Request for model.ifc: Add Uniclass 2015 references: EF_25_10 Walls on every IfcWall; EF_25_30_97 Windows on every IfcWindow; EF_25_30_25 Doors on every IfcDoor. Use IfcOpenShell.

First a look at what the model holds.

```python
import ifcopenshell

model = ifcopenshell.open("model.ifc")
print(model.schema)
print("classifications:", [c.Name for c in model.by_type("IfcClassification")])
for ifc_class in ("IfcDoor", "IfcRoof", "IfcStair", "IfcWall", "IfcWindow"):
    print(ifc_class, len(model.by_type(ifc_class)))
```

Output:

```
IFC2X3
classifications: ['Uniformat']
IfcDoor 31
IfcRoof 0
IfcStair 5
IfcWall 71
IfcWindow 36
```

```python
import ifcopenshell
import ifcopenshell.api.classification

model = ifcopenshell.open("model.ifc")

# IFC2X3 requires Source and Edition and has no link from the project to the system.
system = model.create_entity("IfcClassification", Source="NBS", Edition="2015", Name="Uniclass 2015")

codes = {
    "IfcWall": ("EF_25_10", "Walls"),
    "IfcWindow": ("EF_25_30_97", "Windows"),
    "IfcDoor": ("EF_25_30_25", "Doors"),
}
for ifc_class, (code, name) in codes.items():
    products = model.by_type(ifc_class)
    ifcopenshell.api.classification.add_reference(
        model, products=products, classification=system, identification=code, name=name
    )
    print(code, len(products))

model.write("model_updated.ifc")
```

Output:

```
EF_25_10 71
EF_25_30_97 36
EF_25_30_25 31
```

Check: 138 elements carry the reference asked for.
